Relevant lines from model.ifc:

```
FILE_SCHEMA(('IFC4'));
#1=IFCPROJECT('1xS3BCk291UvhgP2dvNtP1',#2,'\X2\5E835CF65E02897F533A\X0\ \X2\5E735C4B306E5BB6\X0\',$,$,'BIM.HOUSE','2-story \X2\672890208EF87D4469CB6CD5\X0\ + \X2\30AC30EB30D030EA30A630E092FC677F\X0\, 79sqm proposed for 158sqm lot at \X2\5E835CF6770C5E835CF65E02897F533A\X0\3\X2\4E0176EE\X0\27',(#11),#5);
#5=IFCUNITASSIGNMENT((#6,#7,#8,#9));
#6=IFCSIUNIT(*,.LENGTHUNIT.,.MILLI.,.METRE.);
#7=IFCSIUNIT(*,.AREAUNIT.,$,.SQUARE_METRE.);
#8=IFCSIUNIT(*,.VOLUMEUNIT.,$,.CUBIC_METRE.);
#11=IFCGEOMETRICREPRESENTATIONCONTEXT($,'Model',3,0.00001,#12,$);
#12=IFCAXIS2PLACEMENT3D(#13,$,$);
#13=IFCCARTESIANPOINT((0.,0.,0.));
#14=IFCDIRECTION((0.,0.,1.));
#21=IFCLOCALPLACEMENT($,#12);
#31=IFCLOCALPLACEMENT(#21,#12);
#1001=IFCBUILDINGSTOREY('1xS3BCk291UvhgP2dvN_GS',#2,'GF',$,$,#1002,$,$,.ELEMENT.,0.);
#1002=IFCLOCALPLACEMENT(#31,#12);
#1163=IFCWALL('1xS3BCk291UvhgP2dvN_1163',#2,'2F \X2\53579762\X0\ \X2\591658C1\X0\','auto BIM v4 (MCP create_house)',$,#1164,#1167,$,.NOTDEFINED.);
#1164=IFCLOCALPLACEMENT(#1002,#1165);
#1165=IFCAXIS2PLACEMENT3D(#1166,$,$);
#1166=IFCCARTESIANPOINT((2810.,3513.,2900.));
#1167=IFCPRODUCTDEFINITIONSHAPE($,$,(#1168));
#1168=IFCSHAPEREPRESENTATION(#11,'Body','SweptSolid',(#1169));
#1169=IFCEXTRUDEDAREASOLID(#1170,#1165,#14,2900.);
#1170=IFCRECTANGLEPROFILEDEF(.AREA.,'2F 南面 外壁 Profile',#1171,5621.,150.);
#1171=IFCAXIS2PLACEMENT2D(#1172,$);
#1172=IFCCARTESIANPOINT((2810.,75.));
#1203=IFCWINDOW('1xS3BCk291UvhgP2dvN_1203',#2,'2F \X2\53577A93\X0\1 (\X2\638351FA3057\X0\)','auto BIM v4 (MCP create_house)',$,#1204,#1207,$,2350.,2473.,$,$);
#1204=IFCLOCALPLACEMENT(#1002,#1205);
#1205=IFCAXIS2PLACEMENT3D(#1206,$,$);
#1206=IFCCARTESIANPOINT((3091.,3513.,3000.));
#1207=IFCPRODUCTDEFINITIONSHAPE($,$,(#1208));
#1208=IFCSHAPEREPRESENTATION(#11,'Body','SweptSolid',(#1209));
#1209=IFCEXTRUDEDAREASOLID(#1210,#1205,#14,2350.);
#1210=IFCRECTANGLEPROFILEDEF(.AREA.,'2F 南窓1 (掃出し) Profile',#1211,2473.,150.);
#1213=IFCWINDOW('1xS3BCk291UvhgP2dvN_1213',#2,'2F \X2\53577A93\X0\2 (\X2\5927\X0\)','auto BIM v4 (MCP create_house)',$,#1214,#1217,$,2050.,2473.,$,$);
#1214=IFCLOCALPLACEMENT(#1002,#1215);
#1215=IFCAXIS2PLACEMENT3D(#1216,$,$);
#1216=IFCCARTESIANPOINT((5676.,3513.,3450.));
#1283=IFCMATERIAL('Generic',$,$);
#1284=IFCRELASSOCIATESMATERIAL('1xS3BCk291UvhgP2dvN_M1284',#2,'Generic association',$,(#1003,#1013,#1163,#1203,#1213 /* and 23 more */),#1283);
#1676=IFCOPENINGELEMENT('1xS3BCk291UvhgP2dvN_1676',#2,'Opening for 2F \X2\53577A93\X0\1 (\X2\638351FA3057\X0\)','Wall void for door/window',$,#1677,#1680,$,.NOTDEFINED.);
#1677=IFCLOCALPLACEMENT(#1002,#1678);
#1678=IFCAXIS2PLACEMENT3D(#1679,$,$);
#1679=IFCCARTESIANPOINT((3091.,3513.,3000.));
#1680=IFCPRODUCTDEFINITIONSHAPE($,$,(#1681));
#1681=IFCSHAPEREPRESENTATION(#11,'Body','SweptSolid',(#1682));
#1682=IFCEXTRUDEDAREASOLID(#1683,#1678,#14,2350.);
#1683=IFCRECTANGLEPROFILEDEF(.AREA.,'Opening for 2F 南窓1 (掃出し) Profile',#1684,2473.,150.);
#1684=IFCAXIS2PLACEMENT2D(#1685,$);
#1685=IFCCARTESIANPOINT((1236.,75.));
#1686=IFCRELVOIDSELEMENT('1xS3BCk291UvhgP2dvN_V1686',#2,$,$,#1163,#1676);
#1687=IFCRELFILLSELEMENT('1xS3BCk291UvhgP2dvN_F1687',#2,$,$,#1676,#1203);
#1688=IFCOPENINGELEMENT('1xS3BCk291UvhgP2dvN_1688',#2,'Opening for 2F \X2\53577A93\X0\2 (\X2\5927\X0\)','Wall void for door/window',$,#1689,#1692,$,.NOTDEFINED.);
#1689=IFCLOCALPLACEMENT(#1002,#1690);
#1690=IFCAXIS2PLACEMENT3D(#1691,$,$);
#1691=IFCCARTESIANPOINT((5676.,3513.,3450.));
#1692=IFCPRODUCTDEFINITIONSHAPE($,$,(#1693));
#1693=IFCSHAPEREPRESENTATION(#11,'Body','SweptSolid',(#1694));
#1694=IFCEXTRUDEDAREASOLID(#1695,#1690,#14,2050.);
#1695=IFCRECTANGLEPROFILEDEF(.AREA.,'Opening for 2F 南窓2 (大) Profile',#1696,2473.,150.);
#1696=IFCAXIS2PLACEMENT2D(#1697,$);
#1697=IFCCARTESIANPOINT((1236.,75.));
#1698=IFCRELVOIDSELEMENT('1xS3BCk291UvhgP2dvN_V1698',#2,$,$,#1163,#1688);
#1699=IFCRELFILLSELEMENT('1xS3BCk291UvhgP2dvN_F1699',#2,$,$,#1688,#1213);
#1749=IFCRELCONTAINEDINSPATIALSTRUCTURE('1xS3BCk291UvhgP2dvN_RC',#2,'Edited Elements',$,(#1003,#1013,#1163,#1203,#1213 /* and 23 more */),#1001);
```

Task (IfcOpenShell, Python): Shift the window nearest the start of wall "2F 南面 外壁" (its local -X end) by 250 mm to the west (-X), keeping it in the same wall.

```python
import ifcopenshell
import ifcopenshell.api.geometry
import ifcopenshell.util.placement

model = ifcopenshell.open("model.ifc")

window = model.by_guid("1xS3BCk291UvhgP2dvN_1203")
opening = window.FillsVoids[0].RelatingOpeningElement
wall = opening.VoidsElements[0].RelatingBuildingElement

wall_matrix = ifcopenshell.util.placement.get_local_placement(wall.ObjectPlacement)
shift = wall_matrix[:3, 0] * -250.0
before = ifcopenshell.util.placement.get_local_placement(window.ObjectPlacement)[:3, 3].copy()

# The window is not placed relative to its opening, so move both.
for product in (opening, window):
    matrix = ifcopenshell.util.placement.get_local_placement(product.ObjectPlacement)
    matrix[:3, 3] += shift
    ifcopenshell.api.geometry.edit_object_placement(model, product=product, matrix=matrix, is_si=False)

after = ifcopenshell.util.placement.get_local_placement(window.ObjectPlacement)[:3, 3]
print("window moved by", (after - before).round(3) + 0.0)

model.write("model_updated.ifc")
```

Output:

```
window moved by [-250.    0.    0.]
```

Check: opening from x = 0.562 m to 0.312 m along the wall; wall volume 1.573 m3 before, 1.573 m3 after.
